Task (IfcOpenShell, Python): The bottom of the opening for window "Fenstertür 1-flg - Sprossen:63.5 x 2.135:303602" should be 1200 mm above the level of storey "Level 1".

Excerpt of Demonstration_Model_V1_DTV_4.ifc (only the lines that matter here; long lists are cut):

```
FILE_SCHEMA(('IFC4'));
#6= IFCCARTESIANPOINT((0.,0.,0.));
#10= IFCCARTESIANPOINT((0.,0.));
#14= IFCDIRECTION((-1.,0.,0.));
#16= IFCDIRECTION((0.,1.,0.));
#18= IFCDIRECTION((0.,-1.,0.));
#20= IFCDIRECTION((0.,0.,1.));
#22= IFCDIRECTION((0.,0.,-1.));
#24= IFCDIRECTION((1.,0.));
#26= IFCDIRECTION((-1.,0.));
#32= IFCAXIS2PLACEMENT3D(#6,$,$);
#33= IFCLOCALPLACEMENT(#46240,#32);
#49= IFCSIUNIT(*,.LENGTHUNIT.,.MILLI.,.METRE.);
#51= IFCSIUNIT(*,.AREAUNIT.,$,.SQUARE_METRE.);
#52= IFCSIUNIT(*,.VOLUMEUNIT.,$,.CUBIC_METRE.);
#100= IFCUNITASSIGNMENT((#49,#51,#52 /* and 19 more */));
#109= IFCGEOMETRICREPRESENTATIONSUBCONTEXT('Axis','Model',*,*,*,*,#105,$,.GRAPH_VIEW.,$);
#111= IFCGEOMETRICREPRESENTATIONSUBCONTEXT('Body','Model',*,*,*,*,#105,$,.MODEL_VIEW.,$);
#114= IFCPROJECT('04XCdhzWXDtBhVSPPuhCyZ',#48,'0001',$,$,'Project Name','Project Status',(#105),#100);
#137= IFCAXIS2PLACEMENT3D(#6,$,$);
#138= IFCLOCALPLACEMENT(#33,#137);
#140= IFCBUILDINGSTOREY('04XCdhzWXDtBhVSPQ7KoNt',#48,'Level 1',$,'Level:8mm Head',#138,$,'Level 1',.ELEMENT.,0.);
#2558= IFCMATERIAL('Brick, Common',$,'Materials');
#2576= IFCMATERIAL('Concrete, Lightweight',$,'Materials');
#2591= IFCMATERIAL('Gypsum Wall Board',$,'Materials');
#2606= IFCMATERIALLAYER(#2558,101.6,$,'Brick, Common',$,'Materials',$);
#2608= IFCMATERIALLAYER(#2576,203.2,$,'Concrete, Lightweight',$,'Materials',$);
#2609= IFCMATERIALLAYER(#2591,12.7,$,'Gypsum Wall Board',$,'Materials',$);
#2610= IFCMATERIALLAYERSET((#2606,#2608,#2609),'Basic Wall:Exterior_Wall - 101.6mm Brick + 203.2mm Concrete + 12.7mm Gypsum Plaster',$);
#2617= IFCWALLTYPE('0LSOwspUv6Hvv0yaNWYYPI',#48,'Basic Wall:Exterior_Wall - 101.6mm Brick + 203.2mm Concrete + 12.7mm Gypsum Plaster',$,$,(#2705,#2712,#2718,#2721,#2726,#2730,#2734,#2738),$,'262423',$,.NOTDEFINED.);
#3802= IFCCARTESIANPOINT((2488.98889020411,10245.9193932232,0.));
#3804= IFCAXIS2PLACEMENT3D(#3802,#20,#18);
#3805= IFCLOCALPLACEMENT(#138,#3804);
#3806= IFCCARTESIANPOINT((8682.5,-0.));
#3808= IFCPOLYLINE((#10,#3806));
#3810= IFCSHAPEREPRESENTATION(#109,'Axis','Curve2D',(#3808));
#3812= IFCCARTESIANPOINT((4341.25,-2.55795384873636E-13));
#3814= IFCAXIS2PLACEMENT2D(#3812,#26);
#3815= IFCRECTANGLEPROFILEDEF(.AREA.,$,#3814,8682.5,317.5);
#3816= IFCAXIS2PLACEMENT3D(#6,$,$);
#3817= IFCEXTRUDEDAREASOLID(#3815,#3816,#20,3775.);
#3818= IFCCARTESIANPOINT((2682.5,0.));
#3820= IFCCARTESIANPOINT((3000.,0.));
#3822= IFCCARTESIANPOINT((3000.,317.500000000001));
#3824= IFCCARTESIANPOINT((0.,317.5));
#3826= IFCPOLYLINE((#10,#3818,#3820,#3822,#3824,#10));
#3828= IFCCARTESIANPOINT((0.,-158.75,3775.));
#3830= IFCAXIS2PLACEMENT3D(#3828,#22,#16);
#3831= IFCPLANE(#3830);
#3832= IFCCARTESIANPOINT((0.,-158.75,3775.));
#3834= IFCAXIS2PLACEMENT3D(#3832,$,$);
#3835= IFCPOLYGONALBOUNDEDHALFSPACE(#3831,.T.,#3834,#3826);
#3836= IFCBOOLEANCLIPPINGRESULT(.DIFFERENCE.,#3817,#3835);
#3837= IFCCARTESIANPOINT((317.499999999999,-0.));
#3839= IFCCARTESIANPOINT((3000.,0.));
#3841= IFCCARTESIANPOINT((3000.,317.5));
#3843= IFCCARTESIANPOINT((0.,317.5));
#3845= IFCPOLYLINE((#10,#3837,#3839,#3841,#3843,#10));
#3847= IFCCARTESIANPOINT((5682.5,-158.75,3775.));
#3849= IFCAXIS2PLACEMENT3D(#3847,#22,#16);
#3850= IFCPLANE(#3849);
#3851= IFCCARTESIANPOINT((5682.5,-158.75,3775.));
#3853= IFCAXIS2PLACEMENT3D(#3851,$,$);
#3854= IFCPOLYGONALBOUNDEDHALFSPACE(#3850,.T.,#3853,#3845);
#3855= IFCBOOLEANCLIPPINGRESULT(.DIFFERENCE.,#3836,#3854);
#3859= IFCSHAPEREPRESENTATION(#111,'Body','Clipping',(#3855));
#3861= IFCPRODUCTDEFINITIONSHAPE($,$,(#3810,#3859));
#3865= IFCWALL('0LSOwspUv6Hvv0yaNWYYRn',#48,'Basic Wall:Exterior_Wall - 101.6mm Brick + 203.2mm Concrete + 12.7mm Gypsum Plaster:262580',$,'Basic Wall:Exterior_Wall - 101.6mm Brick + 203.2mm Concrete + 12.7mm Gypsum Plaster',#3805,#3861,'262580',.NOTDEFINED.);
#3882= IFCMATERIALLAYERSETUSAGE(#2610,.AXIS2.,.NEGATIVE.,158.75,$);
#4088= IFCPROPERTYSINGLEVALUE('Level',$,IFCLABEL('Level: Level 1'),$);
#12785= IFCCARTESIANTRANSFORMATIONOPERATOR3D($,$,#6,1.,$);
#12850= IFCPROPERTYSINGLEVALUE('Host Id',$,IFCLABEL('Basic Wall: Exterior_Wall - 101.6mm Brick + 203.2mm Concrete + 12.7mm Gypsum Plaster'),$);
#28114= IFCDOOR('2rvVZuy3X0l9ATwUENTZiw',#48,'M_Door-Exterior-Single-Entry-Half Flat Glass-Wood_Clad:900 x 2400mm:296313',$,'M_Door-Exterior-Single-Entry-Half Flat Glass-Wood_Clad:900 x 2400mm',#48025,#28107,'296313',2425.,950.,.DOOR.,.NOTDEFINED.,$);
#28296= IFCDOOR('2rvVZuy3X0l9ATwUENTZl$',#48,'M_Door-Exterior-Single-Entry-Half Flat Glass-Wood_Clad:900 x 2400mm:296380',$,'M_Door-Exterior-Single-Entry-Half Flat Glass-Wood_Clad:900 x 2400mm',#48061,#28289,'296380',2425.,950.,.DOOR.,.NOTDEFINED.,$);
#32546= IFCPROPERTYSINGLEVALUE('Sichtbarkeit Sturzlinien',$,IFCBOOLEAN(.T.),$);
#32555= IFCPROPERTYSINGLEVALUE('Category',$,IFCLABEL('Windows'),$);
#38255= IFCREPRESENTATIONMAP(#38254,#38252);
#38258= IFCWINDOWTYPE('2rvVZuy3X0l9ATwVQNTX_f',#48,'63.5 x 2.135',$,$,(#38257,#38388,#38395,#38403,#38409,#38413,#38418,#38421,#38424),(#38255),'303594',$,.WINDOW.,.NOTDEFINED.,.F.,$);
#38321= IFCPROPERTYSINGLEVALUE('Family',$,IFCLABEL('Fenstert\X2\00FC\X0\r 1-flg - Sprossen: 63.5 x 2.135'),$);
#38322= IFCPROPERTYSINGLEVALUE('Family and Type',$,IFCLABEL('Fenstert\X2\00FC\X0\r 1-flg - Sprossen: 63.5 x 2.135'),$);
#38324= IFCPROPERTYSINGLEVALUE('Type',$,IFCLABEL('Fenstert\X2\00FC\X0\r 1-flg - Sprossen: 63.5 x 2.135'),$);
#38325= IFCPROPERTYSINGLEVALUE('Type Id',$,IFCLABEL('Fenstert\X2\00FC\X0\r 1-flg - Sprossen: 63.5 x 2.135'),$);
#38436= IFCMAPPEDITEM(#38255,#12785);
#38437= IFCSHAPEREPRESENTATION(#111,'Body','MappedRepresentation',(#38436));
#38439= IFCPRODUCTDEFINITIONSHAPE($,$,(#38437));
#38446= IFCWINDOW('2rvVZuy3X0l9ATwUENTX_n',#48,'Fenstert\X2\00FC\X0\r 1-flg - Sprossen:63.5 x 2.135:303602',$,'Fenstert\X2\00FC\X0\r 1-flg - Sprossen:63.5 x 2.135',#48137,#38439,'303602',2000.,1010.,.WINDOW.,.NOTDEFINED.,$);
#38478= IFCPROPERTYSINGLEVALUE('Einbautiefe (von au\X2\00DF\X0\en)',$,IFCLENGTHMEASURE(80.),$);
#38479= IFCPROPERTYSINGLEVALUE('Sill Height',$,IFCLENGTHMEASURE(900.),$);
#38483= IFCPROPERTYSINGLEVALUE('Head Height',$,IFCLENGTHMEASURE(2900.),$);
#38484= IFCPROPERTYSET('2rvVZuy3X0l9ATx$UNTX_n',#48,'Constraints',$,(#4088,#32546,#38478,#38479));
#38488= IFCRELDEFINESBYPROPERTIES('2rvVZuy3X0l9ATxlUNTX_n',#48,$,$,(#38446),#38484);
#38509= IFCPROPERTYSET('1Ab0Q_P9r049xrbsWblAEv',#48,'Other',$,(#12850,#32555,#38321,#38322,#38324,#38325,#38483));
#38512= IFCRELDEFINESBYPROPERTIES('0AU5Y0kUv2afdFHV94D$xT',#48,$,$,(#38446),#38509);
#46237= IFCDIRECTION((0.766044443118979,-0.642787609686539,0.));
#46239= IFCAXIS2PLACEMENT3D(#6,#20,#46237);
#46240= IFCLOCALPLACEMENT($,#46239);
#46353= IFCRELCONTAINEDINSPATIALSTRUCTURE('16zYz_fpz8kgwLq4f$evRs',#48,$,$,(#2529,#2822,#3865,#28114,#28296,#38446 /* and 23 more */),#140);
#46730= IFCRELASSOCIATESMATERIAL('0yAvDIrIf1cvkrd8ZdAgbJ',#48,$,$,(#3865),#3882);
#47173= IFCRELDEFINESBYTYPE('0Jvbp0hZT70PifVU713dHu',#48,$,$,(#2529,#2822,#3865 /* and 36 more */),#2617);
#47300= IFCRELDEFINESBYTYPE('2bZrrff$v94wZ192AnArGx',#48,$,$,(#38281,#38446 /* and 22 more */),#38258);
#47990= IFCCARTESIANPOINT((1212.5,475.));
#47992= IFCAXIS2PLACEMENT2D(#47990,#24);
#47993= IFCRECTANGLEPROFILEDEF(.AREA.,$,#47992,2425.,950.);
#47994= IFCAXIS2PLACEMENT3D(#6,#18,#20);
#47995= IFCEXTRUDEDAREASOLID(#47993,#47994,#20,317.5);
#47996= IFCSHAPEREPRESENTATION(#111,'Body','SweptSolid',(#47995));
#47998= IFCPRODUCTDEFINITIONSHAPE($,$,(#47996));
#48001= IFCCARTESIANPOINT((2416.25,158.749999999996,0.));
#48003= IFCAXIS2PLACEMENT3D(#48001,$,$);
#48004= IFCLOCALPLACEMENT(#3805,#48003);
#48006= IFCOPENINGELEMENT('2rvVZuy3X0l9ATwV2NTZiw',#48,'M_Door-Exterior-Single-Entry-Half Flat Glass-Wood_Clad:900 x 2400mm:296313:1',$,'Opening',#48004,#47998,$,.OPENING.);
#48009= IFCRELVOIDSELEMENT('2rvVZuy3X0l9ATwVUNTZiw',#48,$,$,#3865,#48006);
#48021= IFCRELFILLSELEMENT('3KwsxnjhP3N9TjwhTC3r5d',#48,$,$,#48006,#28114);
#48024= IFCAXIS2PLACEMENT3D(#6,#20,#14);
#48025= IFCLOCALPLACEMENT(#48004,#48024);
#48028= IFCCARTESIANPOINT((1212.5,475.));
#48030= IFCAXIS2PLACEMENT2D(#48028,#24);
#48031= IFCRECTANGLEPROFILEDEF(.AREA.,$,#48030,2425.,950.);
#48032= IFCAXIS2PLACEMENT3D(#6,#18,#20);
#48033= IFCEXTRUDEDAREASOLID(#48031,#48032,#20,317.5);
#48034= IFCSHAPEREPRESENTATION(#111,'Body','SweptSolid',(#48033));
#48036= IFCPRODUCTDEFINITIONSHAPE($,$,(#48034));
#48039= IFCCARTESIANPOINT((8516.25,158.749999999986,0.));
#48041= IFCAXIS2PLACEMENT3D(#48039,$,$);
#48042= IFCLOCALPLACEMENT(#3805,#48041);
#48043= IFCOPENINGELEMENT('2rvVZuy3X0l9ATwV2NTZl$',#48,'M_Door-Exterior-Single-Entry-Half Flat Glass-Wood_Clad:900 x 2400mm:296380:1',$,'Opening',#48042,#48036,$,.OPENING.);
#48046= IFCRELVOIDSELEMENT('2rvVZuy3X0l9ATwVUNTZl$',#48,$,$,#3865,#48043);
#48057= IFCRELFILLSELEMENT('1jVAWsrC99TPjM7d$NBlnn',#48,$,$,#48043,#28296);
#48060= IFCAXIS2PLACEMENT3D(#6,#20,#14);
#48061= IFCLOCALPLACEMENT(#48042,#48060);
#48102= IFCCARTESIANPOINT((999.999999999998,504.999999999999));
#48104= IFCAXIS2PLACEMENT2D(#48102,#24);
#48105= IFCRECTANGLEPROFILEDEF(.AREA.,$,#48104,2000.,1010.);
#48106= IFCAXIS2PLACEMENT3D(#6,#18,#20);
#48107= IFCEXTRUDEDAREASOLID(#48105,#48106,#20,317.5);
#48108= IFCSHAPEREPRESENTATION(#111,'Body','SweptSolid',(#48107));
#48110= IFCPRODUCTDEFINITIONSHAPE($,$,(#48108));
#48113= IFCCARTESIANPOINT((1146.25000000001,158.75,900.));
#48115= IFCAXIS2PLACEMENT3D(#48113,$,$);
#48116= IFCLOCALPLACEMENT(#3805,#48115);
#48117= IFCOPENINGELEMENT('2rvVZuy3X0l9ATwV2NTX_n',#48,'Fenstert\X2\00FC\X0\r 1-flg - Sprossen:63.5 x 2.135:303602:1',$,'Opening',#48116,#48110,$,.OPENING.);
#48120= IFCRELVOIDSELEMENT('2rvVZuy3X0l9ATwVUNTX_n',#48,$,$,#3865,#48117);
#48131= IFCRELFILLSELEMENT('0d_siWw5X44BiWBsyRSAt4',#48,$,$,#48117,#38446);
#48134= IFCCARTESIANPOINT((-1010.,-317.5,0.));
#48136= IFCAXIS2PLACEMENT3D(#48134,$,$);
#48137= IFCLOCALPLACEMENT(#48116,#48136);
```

```python
import numpy as np
import ifcopenshell
import ifcopenshell.api.geometry
import ifcopenshell.api.pset
import ifcopenshell.geom
import ifcopenshell.util.element
import ifcopenshell.util.placement
import ifcopenshell.util.shape
import ifcopenshell.util.unit

model = ifcopenshell.open("Demonstration_Model_V1_DTV_4.ifc")
unit_scale = ifcopenshell.util.unit.calculate_unit_scale(model)

window = model.by_guid("2rvVZuy3X0l9ATwUENTX_n")
opening = window.FillsVoids[0].RelatingOpeningElement
storey = ifcopenshell.util.element.get_container(window, ifc_class="IfcBuildingStorey")
level = ifcopenshell.util.placement.get_local_placement(storey.ObjectPlacement)[2, 3]

# The opening's origin need not be at the sill, so measure its lowest point.
shape = ifcopenshell.geom.create_shape(ifcopenshell.geom.settings(), opening)
bottom = ifcopenshell.util.shape.get_shape_bottom_elevation(shape, shape.geometry) / unit_scale
dz = level + 1.2 / unit_scale - bottom

shift = np.array([0.0, 0.0, dz])
# The window is placed relative to its opening, so it follows when the opening moves.
matrix = ifcopenshell.util.placement.get_local_placement(opening.ObjectPlacement)
matrix[:3, 3] += shift
ifcopenshell.api.geometry.edit_object_placement(
    model, product=opening, matrix=matrix, is_si=False, should_transform_children=True
)

# Keep the stored heights in step.
pset = model.by_id(ifcopenshell.util.element.get_pset(window, "Constraints", should_inherit=False)["id"])
ifcopenshell.api.pset.edit_pset(model, pset=pset, properties={
    "Sill Height": model.create_entity("IfcLengthMeasure", ifcopenshell.util.element.get_pset(window, "Constraints", "Sill Height") + dz),
})
pset = model.by_id(ifcopenshell.util.element.get_pset(window, "Other", should_inherit=False)["id"])
ifcopenshell.api.pset.edit_pset(model, pset=pset, properties={
    "Head Height": model.create_entity("IfcLengthMeasure", ifcopenshell.util.element.get_pset(window, "Other", "Head Height") + dz),
})

print(f"moved by {dz * unit_scale:+.3f} m")

model.write("Demonstration_Model_V1_DTV_4_edited.ifc")
```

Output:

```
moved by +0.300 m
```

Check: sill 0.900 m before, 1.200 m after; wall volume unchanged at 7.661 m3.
